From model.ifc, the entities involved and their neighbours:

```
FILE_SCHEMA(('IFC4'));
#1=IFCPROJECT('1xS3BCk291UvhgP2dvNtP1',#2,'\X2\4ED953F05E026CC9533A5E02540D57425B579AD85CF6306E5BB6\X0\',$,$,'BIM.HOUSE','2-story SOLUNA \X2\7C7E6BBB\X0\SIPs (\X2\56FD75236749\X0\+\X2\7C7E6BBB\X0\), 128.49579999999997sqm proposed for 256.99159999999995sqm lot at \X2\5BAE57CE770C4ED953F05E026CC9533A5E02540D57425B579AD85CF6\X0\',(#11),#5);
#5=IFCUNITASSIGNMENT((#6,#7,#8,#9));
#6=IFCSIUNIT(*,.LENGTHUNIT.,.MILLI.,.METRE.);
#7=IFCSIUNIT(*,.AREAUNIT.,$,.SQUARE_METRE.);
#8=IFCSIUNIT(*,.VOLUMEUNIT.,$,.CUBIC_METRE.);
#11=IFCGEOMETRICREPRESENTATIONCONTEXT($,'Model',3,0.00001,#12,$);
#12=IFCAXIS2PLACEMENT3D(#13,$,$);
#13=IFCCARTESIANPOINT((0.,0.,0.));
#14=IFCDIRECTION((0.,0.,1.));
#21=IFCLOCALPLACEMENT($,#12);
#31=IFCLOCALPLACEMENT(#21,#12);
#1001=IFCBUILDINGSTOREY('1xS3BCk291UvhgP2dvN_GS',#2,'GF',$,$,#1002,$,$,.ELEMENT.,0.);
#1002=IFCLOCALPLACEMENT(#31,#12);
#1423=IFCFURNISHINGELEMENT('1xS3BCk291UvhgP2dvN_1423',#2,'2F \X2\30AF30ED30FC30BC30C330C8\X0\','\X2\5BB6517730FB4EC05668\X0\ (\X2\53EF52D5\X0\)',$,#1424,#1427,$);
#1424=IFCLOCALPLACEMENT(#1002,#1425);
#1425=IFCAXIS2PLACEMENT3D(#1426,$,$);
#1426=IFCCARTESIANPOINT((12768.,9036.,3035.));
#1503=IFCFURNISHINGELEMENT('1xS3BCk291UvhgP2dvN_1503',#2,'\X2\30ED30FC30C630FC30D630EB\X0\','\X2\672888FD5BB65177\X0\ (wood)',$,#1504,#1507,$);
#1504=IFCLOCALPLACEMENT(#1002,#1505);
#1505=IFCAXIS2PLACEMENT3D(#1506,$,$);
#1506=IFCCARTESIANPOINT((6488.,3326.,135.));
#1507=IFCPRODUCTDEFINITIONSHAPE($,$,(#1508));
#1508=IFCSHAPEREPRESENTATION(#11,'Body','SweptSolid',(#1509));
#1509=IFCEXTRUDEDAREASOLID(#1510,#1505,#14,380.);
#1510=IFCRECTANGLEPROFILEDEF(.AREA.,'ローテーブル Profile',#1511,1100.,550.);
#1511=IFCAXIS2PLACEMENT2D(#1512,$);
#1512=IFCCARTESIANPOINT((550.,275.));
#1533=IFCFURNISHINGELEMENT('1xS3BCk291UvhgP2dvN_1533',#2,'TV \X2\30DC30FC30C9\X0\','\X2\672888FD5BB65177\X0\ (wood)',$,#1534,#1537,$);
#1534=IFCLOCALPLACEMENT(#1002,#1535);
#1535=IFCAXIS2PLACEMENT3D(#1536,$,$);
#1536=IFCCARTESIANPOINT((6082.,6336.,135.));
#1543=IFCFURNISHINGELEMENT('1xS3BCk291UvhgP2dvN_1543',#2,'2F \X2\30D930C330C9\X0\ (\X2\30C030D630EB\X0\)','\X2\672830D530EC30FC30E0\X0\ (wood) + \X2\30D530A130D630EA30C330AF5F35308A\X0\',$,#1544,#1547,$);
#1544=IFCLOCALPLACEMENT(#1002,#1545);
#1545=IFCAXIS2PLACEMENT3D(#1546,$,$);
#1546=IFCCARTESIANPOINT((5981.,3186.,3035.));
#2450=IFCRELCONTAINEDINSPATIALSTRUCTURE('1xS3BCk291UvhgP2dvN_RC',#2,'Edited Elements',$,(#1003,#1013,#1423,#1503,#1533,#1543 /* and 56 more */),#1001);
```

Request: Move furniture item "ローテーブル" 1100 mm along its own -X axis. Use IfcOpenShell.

```python
import ifcopenshell
import ifcopenshell.api.geometry
import ifcopenshell.util.placement

model = ifcopenshell.open("model.ifc")

item = model.by_id(1503)
matrix = ifcopenshell.util.placement.get_local_placement(item.ObjectPlacement)
matrix[:3, 3] -= matrix[:3, 0] * 1100.0
ifcopenshell.api.geometry.edit_object_placement(model, product=item, matrix=matrix, is_si=False)

print(ifcopenshell.util.placement.get_local_placement(item.ObjectPlacement).round(3) + 0.0)

model.write("model_v2.ifc")
```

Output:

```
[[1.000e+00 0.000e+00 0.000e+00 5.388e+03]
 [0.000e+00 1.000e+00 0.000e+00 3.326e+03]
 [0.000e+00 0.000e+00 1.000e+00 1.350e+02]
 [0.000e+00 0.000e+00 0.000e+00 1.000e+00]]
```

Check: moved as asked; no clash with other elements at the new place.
